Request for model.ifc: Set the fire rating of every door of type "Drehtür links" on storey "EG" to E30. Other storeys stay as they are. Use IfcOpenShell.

First a look at what the model holds.

```python
import ifcopenshell
import ifcopenshell.util.element

model = ifcopenshell.open("model.ifc")
print(model.schema)
storey = next(s for s in model.by_type("IfcBuildingStorey") if s.Name == "EG")
doors = [e for e in ifcopenshell.util.element.get_decomposition(storey) if e.is_a("IfcDoor")]
seen = {}
for e in doors:
    element_type = ifcopenshell.util.element.get_type(e)
    key = (element_type.Name if element_type != e and element_type else None, ifcopenshell.util.element.get_pset(e, "Pset_DoorCommon", "FireRating"))
    seen[key] = seen.get(key, 0) + 1
for (name, value), count in sorted(seen.items(), key=str):
    print(count, "x", name, "|", value)
```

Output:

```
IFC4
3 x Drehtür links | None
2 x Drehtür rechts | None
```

```python
import ifcopenshell
import ifcopenshell.api.pset
import ifcopenshell.util.element

model = ifcopenshell.open("model.ifc")

storey = next(s for s in model.by_type("IfcBuildingStorey") if s.Name == "EG")
doors = [e for e in ifcopenshell.util.element.get_decomposition(storey) if e.is_a("IfcDoor")]

count = 0
for e in doors:
    element_type = ifcopenshell.util.element.get_type(e)
    if element_type in (None, e) or element_type.Name != "Drehtür links":
        continue
    # add_pset returns the element's existing set when there is one.
    pset = ifcopenshell.api.pset.add_pset(model, product=e, name="Pset_DoorCommon")
    ifcopenshell.api.pset.edit_pset(model, pset=pset, properties={"FireRating": "E30"})
    count += 1

print(count, "doors updated")

model.write("model-out.ifc")
```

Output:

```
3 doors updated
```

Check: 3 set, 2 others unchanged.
